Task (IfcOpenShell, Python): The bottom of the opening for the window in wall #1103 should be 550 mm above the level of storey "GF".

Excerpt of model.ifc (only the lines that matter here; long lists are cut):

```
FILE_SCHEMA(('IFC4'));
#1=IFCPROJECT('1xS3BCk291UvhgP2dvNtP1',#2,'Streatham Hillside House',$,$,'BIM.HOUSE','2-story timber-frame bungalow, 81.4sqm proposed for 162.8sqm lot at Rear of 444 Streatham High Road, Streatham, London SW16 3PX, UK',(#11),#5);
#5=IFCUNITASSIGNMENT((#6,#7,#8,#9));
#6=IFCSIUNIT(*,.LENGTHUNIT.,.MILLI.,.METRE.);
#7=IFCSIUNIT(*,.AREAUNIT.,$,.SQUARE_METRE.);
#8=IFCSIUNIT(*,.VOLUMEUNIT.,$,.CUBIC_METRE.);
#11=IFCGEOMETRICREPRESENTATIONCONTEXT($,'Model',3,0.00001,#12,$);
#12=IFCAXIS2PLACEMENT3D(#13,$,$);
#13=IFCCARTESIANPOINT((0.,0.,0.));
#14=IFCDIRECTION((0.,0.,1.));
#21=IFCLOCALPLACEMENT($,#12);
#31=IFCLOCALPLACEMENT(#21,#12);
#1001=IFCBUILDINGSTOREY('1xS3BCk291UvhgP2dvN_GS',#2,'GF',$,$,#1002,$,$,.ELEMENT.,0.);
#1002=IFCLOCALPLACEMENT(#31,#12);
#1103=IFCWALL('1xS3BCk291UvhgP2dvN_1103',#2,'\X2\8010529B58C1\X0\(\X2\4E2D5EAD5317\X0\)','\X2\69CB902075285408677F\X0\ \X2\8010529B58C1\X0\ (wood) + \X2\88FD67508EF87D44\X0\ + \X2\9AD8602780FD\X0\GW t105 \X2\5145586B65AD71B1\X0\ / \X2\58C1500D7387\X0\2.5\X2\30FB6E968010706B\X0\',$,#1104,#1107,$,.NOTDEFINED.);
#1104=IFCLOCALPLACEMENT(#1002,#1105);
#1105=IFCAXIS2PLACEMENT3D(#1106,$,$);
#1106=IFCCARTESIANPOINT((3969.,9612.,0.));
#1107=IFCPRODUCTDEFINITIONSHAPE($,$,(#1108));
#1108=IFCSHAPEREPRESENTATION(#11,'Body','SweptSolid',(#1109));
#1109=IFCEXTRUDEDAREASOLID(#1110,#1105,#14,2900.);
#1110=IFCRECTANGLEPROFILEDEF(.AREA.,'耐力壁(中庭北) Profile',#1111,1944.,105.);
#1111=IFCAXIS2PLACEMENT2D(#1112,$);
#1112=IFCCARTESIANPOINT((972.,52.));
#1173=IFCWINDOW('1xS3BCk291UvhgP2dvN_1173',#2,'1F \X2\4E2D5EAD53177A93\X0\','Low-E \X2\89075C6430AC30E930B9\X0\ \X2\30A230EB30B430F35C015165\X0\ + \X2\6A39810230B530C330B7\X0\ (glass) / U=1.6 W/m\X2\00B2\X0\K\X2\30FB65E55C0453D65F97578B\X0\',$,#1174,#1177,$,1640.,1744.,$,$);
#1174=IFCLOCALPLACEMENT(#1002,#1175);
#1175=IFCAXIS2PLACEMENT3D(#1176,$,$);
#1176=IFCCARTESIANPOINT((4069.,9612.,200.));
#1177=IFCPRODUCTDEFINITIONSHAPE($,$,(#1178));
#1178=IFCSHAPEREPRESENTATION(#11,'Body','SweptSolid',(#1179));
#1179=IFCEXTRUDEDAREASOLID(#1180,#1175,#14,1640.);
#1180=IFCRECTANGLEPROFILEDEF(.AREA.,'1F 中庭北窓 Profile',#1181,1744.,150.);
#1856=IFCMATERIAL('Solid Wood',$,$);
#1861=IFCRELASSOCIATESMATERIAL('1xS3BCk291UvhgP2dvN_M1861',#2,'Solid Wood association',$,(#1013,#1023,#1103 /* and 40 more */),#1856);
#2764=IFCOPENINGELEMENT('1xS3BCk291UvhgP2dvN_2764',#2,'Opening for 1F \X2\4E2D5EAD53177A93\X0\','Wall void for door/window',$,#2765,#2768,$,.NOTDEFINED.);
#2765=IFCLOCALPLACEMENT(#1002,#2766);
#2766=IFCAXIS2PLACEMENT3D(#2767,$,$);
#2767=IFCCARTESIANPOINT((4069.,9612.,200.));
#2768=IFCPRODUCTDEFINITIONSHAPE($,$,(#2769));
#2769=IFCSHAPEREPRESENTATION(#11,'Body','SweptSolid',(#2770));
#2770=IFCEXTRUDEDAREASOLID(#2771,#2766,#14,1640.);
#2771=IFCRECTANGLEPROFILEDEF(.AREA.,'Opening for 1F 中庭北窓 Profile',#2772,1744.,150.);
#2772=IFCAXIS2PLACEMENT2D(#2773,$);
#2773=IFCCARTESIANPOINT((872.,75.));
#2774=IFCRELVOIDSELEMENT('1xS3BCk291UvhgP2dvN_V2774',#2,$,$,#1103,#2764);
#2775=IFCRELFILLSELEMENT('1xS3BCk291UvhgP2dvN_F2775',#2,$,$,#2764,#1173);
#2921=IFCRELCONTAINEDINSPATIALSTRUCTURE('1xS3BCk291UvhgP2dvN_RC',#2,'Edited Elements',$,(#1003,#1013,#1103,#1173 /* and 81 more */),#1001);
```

```python
import numpy as np
import ifcopenshell
import ifcopenshell.api.geometry
import ifcopenshell.geom
import ifcopenshell.util.element
import ifcopenshell.util.placement
import ifcopenshell.util.shape
import ifcopenshell.util.unit

model = ifcopenshell.open("model.ifc")
unit_scale = ifcopenshell.util.unit.calculate_unit_scale(model)

window = model.by_guid("1xS3BCk291UvhgP2dvN_1173")
opening = window.FillsVoids[0].RelatingOpeningElement
storey = ifcopenshell.util.element.get_container(window, ifc_class="IfcBuildingStorey")
level = ifcopenshell.util.placement.get_local_placement(storey.ObjectPlacement)[2, 3]

# The opening's origin need not be at the sill, so measure its lowest point.
shape = ifcopenshell.geom.create_shape(ifcopenshell.geom.settings(), opening)
bottom = ifcopenshell.util.shape.get_shape_bottom_elevation(shape, shape.geometry) / unit_scale
dz = level + 0.55 / unit_scale - bottom

shift = np.array([0.0, 0.0, dz])
# The window is not placed relative to its opening, so move both.
for product in (opening, window):
    matrix = ifcopenshell.util.placement.get_local_placement(product.ObjectPlacement)
    matrix[:3, 3] += shift
    ifcopenshell.api.geometry.edit_object_placement(model, product=product, matrix=matrix, is_si=False)

print(f"moved by {dz * unit_scale:+.3f} m")

model.write("model-out.ifc")
```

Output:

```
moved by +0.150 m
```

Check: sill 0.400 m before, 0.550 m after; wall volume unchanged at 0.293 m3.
